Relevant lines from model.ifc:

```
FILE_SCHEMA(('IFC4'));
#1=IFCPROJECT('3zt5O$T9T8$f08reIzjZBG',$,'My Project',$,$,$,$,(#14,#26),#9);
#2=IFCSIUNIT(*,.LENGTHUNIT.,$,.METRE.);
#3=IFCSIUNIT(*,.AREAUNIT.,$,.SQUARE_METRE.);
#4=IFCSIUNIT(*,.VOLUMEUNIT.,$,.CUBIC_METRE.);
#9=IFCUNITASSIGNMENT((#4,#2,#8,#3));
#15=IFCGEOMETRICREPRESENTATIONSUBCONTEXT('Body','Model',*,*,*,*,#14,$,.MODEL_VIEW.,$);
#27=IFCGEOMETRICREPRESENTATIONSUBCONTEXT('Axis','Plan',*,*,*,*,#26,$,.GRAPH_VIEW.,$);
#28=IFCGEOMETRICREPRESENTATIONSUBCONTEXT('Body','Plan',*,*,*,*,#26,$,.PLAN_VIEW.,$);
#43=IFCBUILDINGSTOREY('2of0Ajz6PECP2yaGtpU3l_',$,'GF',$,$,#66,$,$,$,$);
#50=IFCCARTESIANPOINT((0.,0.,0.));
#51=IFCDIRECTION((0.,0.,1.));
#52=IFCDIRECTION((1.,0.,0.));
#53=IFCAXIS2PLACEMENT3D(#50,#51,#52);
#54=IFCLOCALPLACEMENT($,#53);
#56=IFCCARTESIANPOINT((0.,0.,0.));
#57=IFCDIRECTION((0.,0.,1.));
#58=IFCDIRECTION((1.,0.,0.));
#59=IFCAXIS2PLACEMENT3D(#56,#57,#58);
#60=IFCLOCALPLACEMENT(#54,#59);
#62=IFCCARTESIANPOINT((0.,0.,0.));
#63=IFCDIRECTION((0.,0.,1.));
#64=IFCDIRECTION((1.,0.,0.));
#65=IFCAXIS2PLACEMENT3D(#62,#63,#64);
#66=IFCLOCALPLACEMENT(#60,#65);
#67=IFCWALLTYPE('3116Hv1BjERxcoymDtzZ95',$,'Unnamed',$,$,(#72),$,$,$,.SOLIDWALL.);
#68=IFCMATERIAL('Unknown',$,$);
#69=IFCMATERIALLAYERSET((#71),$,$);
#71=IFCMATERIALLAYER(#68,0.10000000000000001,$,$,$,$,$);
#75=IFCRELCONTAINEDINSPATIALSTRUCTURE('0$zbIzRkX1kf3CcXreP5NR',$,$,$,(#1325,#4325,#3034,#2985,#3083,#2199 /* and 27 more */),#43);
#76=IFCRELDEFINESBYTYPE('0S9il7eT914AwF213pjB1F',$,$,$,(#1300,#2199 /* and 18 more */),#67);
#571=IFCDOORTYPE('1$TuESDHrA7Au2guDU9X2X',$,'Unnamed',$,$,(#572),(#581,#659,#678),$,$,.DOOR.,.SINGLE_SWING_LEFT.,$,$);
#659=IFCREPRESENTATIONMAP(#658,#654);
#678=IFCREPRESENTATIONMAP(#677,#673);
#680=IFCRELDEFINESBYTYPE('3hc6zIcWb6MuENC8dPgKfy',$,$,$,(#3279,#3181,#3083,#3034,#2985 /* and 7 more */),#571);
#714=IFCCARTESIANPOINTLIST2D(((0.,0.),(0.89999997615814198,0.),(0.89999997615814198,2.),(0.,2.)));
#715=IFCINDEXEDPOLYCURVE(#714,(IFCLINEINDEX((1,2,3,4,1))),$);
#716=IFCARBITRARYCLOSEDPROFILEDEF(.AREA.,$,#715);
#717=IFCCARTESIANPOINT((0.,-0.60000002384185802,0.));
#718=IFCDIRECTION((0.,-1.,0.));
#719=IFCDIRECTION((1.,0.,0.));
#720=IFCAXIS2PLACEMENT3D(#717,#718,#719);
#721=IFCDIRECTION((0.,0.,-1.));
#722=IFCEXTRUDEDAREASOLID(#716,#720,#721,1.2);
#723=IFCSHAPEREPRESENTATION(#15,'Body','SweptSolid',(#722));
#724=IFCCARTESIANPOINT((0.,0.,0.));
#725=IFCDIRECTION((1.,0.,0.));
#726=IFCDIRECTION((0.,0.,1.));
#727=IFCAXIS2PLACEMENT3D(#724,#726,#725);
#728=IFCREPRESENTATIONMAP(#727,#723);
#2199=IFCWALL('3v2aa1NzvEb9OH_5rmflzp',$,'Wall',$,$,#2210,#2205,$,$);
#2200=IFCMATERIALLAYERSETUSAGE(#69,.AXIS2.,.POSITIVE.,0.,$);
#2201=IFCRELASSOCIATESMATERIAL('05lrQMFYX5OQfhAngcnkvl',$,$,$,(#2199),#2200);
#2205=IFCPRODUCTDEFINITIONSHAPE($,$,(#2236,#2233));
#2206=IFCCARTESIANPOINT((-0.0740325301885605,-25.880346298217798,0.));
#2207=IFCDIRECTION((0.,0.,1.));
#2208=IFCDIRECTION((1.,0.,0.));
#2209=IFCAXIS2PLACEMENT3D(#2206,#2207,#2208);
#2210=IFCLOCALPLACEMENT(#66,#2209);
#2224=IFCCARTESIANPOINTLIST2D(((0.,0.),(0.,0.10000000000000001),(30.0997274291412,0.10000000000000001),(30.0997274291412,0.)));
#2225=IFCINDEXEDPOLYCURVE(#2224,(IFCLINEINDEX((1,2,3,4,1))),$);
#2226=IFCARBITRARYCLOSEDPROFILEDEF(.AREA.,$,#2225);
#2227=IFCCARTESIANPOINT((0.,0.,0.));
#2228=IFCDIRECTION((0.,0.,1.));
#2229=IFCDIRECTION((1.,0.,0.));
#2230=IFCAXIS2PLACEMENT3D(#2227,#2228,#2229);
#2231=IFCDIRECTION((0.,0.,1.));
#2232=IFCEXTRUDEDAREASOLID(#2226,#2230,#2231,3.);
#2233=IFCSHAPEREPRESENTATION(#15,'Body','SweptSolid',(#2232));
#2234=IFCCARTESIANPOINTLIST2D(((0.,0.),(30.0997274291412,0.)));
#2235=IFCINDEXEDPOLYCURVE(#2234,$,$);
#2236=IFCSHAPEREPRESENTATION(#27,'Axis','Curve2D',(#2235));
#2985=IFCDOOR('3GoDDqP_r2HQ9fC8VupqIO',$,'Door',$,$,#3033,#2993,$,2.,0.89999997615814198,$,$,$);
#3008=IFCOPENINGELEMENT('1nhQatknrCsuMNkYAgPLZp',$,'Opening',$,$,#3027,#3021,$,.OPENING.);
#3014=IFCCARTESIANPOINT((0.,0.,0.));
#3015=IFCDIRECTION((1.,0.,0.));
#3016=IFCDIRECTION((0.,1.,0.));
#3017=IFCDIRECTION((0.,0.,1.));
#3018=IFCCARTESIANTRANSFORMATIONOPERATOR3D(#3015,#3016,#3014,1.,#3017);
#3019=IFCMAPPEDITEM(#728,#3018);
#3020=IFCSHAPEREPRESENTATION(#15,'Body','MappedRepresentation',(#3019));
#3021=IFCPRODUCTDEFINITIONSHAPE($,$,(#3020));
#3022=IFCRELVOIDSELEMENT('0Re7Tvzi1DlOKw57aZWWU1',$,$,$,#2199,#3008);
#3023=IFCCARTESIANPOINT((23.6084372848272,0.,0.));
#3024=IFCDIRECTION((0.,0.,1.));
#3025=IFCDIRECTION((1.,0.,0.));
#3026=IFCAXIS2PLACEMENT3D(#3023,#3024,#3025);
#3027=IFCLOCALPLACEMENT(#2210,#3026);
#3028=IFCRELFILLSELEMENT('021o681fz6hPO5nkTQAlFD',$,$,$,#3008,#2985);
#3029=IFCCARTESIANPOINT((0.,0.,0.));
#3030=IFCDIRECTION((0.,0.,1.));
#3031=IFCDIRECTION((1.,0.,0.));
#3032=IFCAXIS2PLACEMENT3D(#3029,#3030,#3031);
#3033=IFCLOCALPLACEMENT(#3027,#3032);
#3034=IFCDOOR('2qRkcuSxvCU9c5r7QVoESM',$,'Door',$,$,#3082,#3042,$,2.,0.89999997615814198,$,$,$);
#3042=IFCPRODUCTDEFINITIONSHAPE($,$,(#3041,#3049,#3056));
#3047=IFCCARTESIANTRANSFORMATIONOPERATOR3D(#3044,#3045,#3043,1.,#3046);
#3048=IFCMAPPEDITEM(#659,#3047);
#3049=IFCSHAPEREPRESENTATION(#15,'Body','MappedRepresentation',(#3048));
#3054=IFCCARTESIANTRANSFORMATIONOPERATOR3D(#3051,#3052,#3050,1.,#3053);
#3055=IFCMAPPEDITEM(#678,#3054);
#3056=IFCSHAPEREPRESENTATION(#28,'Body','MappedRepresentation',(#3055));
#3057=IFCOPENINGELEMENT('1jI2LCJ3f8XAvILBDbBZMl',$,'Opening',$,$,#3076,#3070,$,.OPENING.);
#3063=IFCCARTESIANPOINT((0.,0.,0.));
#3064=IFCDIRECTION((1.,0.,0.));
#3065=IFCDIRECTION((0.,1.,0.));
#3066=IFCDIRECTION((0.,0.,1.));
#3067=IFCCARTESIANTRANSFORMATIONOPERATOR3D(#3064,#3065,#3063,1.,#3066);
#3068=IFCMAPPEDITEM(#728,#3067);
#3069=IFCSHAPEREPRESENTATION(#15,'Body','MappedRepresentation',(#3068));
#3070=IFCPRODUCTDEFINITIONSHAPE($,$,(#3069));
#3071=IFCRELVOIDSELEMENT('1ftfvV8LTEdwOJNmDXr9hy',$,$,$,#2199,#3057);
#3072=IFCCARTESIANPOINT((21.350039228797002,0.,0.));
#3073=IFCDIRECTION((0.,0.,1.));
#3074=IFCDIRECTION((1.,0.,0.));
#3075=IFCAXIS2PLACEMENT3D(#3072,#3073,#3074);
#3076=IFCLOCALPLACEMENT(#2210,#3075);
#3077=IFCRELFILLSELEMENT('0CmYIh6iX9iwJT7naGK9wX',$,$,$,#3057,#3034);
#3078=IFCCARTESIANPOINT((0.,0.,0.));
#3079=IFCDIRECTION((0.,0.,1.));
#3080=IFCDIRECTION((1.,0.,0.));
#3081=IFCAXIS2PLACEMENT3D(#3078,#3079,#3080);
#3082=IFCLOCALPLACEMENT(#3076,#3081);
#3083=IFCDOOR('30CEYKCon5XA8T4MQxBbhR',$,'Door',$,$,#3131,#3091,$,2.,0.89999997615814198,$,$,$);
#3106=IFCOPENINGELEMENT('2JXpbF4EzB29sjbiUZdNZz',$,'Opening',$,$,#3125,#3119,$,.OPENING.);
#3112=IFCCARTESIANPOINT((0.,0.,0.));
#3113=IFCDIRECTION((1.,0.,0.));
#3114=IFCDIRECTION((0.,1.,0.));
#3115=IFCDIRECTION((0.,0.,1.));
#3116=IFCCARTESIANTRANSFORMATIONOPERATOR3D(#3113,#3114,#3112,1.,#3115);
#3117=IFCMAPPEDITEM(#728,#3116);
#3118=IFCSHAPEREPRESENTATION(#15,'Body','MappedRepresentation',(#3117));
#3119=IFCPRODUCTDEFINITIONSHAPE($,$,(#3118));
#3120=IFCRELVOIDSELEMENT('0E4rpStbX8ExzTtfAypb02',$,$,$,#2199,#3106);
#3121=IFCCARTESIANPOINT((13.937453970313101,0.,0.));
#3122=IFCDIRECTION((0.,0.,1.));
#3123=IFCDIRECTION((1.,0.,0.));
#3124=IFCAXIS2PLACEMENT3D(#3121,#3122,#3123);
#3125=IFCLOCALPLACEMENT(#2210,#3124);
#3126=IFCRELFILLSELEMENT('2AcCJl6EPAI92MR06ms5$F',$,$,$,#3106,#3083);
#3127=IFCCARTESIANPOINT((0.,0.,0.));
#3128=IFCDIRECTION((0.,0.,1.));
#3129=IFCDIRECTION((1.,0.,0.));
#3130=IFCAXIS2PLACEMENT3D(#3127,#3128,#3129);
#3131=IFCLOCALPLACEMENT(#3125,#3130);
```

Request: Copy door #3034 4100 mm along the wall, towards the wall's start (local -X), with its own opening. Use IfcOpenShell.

```python
import ifcopenshell
import ifcopenshell.api.feature
import ifcopenshell.api.geometry
import ifcopenshell.api.root
import ifcopenshell.geom
import ifcopenshell.util.element
import ifcopenshell.util.placement
import ifcopenshell.util.shape
import ifcopenshell.util.unit

model = ifcopenshell.open("model.ifc")
unit_scale = ifcopenshell.util.unit.calculate_unit_scale(model)
settings = ifcopenshell.geom.settings()


def volume(element):
    """Net volume in cubic metres, openings subtracted."""
    shape = ifcopenshell.geom.create_shape(settings, element)
    return ifcopenshell.util.shape.get_volume(shape.geometry)


door = model.by_id(3034)
opening = door.FillsVoids[0].RelatingOpeningElement
wall = opening.VoidsElements[0].RelatingBuildingElement
before = volume(wall)
shift = ifcopenshell.util.placement.get_local_placement(wall.ObjectPlacement)[:3, 0] * -4.1 / unit_scale

# copy_class copies the void relationship, type, container and properties, but no geometry.
new_opening = ifcopenshell.api.root.copy_class(model, product=opening)
new_opening.Representation = ifcopenshell.util.element.copy_deep(
    model, opening.Representation, exclude=["IfcGeometricRepresentationContext", "IfcRepresentationMap"]
)
new_door = ifcopenshell.api.root.copy_class(model, product=door)
new_door.Representation = ifcopenshell.util.element.copy_deep(
    model, door.Representation, exclude=["IfcGeometricRepresentationContext", "IfcRepresentationMap"]
)
ifcopenshell.api.feature.add_filling(model, opening=new_opening, element=new_door)

for old, new in ((opening, new_opening), (door, new_door)):
    matrix = ifcopenshell.util.placement.get_local_placement(old.ObjectPlacement)
    matrix[:3, 3] += shift
    ifcopenshell.api.geometry.edit_object_placement(model, product=new, matrix=matrix, is_si=False)

after = volume(wall)

print(f"wall volume {before:.3f} -> {after:.3f} m3")

model.write("model-out.ifc")
```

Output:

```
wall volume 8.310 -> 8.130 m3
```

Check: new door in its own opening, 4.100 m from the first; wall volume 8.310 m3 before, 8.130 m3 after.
